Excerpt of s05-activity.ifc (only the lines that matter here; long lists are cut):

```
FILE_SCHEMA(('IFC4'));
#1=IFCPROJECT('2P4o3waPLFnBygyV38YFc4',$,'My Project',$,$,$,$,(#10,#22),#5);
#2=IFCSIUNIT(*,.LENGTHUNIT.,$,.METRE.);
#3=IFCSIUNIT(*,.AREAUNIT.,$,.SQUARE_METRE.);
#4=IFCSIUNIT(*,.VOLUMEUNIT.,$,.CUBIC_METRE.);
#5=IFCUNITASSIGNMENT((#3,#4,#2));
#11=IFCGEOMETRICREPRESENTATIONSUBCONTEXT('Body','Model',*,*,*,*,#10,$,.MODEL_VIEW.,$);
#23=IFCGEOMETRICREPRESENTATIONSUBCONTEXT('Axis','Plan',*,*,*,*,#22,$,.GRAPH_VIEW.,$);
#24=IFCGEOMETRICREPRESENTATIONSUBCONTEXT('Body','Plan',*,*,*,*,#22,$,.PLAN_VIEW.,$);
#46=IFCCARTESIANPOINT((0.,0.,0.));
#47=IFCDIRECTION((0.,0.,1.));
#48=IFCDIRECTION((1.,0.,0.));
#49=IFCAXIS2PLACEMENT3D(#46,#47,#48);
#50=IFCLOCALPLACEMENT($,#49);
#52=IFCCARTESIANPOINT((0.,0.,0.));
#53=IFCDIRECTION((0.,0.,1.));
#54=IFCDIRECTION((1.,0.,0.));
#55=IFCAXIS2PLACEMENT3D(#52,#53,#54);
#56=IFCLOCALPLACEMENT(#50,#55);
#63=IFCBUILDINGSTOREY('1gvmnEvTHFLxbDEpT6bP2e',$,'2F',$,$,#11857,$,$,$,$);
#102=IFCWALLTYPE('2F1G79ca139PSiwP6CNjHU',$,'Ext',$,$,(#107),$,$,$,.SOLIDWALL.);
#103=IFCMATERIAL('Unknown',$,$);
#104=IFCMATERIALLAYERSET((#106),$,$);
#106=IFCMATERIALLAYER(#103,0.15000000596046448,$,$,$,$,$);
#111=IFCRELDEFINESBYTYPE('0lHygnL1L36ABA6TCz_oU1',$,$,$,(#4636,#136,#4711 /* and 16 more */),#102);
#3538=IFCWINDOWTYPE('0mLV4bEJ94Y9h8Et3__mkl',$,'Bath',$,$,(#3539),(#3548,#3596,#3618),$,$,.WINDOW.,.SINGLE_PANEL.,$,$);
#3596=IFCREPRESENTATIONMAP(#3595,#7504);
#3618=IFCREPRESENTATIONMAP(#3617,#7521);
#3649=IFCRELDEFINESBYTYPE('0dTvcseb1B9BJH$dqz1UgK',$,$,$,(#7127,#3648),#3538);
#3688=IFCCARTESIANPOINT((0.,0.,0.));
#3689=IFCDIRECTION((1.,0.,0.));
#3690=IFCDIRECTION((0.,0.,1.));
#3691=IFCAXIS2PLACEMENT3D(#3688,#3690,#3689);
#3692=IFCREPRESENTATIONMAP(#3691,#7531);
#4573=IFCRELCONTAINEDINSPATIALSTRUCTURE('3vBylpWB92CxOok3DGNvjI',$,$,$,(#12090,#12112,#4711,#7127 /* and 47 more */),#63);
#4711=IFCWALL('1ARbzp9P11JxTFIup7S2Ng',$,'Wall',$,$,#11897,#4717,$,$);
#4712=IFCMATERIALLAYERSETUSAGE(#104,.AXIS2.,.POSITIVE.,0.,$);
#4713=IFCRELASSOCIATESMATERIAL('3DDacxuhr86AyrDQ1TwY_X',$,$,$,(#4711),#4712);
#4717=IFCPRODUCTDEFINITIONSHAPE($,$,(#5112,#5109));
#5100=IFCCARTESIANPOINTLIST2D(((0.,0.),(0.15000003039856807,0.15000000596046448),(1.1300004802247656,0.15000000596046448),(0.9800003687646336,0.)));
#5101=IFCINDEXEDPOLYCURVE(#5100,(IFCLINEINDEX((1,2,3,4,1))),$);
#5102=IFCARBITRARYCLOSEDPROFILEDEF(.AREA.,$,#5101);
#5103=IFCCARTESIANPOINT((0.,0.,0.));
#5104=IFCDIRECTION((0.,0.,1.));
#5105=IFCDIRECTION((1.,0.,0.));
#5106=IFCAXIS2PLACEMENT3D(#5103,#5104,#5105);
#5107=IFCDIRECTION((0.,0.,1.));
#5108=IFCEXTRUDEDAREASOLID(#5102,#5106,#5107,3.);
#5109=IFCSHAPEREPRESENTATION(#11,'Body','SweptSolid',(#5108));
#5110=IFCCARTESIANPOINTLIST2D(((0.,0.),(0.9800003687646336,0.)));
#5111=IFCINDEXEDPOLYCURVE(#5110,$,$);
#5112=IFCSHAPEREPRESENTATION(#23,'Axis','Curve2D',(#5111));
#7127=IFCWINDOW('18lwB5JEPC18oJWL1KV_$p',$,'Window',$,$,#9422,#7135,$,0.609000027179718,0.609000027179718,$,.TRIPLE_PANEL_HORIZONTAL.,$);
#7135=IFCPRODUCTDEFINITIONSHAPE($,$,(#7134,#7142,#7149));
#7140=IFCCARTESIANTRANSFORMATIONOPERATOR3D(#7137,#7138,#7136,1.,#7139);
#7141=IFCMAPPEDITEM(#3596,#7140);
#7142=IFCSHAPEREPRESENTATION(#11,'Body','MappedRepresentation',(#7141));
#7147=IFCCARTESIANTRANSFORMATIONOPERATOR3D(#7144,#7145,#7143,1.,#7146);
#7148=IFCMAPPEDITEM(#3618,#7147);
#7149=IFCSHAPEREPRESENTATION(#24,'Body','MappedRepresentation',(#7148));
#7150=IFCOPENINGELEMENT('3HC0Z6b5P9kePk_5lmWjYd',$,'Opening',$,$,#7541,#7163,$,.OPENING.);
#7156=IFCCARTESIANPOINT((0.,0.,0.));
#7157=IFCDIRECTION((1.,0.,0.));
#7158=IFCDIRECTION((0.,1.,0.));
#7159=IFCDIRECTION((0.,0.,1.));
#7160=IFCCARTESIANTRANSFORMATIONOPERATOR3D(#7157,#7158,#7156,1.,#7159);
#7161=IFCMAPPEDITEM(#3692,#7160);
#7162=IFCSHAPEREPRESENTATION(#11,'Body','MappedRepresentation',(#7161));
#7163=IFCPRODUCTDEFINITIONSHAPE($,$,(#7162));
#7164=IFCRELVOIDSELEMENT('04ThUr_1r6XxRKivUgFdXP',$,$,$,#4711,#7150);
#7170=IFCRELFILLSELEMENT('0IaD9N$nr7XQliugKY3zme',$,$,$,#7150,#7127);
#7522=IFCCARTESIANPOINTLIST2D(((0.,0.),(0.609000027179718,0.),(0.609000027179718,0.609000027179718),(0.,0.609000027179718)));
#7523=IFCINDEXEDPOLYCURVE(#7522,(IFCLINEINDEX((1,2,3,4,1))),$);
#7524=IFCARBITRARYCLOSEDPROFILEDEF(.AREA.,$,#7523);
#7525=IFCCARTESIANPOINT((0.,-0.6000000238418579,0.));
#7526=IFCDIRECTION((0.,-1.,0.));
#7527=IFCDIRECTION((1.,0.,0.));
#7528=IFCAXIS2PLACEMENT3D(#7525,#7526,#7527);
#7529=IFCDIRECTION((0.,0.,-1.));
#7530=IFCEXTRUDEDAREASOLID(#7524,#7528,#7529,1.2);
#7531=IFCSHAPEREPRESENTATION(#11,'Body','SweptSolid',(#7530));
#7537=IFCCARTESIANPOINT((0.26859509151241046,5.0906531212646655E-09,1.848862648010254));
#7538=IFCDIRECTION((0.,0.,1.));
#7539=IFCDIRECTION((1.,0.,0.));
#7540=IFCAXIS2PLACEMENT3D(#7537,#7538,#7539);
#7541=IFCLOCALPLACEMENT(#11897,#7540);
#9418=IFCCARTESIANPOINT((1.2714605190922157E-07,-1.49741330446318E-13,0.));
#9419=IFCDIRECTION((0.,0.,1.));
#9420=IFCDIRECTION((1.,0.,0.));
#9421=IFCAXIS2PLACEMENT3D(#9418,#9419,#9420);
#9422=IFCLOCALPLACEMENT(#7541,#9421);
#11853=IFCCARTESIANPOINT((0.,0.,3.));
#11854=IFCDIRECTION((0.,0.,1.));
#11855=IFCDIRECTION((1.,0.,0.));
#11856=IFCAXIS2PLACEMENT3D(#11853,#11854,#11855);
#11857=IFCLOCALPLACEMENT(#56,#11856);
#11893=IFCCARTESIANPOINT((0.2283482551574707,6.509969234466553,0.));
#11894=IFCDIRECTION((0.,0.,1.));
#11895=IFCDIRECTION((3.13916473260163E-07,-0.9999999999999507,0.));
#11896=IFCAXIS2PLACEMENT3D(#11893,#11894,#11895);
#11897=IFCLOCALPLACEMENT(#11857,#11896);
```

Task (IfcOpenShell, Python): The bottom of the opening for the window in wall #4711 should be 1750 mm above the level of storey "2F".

```python
import numpy as np
import ifcopenshell
import ifcopenshell.api.geometry
import ifcopenshell.geom
import ifcopenshell.util.element
import ifcopenshell.util.placement
import ifcopenshell.util.shape
import ifcopenshell.util.unit

model = ifcopenshell.open("s05-activity.ifc")
unit_scale = ifcopenshell.util.unit.calculate_unit_scale(model)

window = model.by_guid("18lwB5JEPC18oJWL1KV_$p")
opening = window.FillsVoids[0].RelatingOpeningElement
storey = ifcopenshell.util.element.get_container(window, ifc_class="IfcBuildingStorey")
level = ifcopenshell.util.placement.get_local_placement(storey.ObjectPlacement)[2, 3]

# The opening's origin need not be at the sill, so measure its lowest point.
shape = ifcopenshell.geom.create_shape(ifcopenshell.geom.settings(), opening)
bottom = ifcopenshell.util.shape.get_shape_bottom_elevation(shape, shape.geometry) / unit_scale
dz = level + 1.75 / unit_scale - bottom

shift = np.array([0.0, 0.0, dz])
# The window is placed relative to its opening, so it follows when the opening moves.
matrix = ifcopenshell.util.placement.get_local_placement(opening.ObjectPlacement)
matrix[:3, 3] += shift
ifcopenshell.api.geometry.edit_object_placement(
    model, product=opening, matrix=matrix, is_si=False, should_transform_children=True
)

print(f"moved by {dz * unit_scale:+.3f} m")

model.write("s05-activity-out.ifc")
```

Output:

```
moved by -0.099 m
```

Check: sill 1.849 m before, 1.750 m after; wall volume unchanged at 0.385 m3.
